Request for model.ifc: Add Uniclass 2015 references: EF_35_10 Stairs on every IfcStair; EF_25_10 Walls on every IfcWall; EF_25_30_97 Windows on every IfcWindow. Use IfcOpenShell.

First a look at what the model holds.

```python
import ifcopenshell

model = ifcopenshell.open("model.ifc")
print(model.schema)
print("classifications:", [c.Name for c in model.by_type("IfcClassification")])
for ifc_class in ("IfcDoor", "IfcRoof", "IfcStair", "IfcWall", "IfcWindow"):
    print(ifc_class, len(model.by_type(ifc_class)))
```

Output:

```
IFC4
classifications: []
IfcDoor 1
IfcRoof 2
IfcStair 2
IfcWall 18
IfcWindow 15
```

```python
import ifcopenshell
import ifcopenshell.api.classification

model = ifcopenshell.open("model.ifc")

system = ifcopenshell.api.classification.add_classification(model, classification="Uniclass 2015")

codes = {
    "IfcStair": ("EF_35_10", "Stairs"),
    "IfcWall": ("EF_25_10", "Walls"),
    "IfcWindow": ("EF_25_30_97", "Windows"),
}
for ifc_class, (code, name) in codes.items():
    products = model.by_type(ifc_class)
    ifcopenshell.api.classification.add_reference(
        model, products=products, classification=system, identification=code, name=name
    )
    print(code, len(products))

model.write("model_updated.ifc")
```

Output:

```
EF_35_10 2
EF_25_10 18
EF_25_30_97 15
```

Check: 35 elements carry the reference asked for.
